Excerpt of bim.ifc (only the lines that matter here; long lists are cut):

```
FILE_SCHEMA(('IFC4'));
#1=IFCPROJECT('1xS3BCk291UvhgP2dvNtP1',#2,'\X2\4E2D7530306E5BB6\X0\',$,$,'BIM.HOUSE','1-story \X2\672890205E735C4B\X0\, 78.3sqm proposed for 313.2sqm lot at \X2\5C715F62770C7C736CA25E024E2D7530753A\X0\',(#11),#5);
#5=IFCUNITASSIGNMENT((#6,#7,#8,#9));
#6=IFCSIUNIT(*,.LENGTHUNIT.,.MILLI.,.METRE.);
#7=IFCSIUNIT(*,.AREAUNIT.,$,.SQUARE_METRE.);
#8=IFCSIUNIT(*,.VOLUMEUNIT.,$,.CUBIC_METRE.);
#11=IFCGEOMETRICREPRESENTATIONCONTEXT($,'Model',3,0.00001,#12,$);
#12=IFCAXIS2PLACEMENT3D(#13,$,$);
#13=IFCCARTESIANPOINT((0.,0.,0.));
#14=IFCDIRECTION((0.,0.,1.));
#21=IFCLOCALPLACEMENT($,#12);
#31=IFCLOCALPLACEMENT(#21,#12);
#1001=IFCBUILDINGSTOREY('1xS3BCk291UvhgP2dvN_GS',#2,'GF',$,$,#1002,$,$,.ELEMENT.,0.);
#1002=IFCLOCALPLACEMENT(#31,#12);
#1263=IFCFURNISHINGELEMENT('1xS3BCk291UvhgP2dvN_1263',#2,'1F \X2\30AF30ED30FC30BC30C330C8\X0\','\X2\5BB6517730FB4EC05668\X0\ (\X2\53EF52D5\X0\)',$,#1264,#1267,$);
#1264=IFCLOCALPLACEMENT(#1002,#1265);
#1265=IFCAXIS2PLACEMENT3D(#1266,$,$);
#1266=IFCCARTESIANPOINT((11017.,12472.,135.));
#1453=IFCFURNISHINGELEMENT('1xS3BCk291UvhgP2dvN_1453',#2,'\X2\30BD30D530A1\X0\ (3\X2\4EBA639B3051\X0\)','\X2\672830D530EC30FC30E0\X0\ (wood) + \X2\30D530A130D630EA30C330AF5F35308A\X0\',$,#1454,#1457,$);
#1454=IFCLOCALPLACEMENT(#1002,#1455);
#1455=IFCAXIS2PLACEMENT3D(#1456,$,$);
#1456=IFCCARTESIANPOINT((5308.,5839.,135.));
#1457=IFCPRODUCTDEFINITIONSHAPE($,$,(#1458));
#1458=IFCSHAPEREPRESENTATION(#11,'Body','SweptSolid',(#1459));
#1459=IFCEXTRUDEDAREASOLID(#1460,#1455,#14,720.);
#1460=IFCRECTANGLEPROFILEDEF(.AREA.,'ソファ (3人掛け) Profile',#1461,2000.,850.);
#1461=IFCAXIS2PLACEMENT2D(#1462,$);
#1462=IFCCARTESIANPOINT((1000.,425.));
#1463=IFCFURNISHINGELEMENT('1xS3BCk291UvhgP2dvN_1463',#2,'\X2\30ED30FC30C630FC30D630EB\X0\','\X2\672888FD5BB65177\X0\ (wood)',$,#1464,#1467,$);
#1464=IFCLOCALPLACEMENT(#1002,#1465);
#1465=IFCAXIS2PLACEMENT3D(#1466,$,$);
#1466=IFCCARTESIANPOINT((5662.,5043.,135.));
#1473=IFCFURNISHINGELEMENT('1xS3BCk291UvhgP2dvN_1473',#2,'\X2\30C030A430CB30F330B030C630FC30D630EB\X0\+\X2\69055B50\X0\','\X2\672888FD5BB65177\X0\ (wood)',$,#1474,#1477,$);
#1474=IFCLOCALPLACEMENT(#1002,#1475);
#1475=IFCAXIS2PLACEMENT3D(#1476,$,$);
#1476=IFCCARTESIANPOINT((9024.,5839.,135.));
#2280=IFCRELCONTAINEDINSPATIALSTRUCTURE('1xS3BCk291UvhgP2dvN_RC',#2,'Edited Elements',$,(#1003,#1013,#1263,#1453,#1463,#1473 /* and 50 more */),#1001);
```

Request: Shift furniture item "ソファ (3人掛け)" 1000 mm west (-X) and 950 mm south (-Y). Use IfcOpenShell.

```python
import ifcopenshell
import ifcopenshell.api.geometry
import ifcopenshell.util.placement

model = ifcopenshell.open("bim.ifc")

item = model.by_id(1453)
matrix = ifcopenshell.util.placement.get_local_placement(item.ObjectPlacement)
matrix[0, 3] -= 1000.0
matrix[1, 3] -= 950.0
ifcopenshell.api.geometry.edit_object_placement(model, product=item, matrix=matrix, is_si=False)

print(ifcopenshell.util.placement.get_local_placement(item.ObjectPlacement).round(3) + 0.0)

model.write("bim_updated.ifc")
```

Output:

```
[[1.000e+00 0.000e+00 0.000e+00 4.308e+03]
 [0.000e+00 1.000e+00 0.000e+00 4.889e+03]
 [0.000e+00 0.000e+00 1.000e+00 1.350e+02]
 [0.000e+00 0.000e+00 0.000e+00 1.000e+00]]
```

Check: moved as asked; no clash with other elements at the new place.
